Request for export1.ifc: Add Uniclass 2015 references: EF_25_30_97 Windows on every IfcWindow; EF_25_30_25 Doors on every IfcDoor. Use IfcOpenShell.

First a look at what the model holds.

```python
import ifcopenshell

model = ifcopenshell.open("export1.ifc")
print(model.schema)
print("classifications:", [c.Name for c in model.by_type("IfcClassification")])
for ifc_class in ("IfcDoor", "IfcRoof", "IfcStair", "IfcWall", "IfcWindow"):
    print(ifc_class, len(model.by_type(ifc_class)))
```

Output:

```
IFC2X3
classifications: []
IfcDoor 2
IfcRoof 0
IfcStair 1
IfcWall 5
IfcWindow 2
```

```python
import ifcopenshell
import ifcopenshell.api.classification

model = ifcopenshell.open("export1.ifc")

# IFC2X3 requires Source and Edition and has no link from the project to the system.
system = model.create_entity("IfcClassification", Source="NBS", Edition="2015", Name="Uniclass 2015")

codes = {
    "IfcWindow": ("EF_25_30_97", "Windows"),
    "IfcDoor": ("EF_25_30_25", "Doors"),
}
for ifc_class, (code, name) in codes.items():
    products = model.by_type(ifc_class)
    ifcopenshell.api.classification.add_reference(
        model, products=products, classification=system, identification=code, name=name
    )
    print(code, len(products))

model.write("export1_updated.ifc")
```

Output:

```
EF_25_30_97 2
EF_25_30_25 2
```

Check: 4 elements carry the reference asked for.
